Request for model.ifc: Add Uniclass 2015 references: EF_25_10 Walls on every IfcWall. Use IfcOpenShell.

First a look at what the model holds.

```python
import ifcopenshell

model = ifcopenshell.open("model.ifc")
print(model.schema)
print("classifications:", [c.Name for c in model.by_type("IfcClassification")])
for ifc_class in ("IfcDoor", "IfcRoof", "IfcStair", "IfcWall", "IfcWindow"):
    print(ifc_class, len(model.by_type(ifc_class)))
```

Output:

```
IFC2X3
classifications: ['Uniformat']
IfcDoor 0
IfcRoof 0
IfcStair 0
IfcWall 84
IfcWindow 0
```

```python
import ifcopenshell
import ifcopenshell.api.classification

model = ifcopenshell.open("model.ifc")

# IFC2X3 requires Source and Edition and has no link from the project to the system.
system = model.create_entity("IfcClassification", Source="NBS", Edition="2015", Name="Uniclass 2015")

codes = {
    "IfcWall": ("EF_25_10", "Walls"),
}
for ifc_class, (code, name) in codes.items():
    products = model.by_type(ifc_class)
    ifcopenshell.api.classification.add_reference(
        model, products=products, classification=system, identification=code, name=name
    )
    print(code, len(products))

model.write("model_rev.ifc")
```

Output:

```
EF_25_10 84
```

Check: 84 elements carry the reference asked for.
